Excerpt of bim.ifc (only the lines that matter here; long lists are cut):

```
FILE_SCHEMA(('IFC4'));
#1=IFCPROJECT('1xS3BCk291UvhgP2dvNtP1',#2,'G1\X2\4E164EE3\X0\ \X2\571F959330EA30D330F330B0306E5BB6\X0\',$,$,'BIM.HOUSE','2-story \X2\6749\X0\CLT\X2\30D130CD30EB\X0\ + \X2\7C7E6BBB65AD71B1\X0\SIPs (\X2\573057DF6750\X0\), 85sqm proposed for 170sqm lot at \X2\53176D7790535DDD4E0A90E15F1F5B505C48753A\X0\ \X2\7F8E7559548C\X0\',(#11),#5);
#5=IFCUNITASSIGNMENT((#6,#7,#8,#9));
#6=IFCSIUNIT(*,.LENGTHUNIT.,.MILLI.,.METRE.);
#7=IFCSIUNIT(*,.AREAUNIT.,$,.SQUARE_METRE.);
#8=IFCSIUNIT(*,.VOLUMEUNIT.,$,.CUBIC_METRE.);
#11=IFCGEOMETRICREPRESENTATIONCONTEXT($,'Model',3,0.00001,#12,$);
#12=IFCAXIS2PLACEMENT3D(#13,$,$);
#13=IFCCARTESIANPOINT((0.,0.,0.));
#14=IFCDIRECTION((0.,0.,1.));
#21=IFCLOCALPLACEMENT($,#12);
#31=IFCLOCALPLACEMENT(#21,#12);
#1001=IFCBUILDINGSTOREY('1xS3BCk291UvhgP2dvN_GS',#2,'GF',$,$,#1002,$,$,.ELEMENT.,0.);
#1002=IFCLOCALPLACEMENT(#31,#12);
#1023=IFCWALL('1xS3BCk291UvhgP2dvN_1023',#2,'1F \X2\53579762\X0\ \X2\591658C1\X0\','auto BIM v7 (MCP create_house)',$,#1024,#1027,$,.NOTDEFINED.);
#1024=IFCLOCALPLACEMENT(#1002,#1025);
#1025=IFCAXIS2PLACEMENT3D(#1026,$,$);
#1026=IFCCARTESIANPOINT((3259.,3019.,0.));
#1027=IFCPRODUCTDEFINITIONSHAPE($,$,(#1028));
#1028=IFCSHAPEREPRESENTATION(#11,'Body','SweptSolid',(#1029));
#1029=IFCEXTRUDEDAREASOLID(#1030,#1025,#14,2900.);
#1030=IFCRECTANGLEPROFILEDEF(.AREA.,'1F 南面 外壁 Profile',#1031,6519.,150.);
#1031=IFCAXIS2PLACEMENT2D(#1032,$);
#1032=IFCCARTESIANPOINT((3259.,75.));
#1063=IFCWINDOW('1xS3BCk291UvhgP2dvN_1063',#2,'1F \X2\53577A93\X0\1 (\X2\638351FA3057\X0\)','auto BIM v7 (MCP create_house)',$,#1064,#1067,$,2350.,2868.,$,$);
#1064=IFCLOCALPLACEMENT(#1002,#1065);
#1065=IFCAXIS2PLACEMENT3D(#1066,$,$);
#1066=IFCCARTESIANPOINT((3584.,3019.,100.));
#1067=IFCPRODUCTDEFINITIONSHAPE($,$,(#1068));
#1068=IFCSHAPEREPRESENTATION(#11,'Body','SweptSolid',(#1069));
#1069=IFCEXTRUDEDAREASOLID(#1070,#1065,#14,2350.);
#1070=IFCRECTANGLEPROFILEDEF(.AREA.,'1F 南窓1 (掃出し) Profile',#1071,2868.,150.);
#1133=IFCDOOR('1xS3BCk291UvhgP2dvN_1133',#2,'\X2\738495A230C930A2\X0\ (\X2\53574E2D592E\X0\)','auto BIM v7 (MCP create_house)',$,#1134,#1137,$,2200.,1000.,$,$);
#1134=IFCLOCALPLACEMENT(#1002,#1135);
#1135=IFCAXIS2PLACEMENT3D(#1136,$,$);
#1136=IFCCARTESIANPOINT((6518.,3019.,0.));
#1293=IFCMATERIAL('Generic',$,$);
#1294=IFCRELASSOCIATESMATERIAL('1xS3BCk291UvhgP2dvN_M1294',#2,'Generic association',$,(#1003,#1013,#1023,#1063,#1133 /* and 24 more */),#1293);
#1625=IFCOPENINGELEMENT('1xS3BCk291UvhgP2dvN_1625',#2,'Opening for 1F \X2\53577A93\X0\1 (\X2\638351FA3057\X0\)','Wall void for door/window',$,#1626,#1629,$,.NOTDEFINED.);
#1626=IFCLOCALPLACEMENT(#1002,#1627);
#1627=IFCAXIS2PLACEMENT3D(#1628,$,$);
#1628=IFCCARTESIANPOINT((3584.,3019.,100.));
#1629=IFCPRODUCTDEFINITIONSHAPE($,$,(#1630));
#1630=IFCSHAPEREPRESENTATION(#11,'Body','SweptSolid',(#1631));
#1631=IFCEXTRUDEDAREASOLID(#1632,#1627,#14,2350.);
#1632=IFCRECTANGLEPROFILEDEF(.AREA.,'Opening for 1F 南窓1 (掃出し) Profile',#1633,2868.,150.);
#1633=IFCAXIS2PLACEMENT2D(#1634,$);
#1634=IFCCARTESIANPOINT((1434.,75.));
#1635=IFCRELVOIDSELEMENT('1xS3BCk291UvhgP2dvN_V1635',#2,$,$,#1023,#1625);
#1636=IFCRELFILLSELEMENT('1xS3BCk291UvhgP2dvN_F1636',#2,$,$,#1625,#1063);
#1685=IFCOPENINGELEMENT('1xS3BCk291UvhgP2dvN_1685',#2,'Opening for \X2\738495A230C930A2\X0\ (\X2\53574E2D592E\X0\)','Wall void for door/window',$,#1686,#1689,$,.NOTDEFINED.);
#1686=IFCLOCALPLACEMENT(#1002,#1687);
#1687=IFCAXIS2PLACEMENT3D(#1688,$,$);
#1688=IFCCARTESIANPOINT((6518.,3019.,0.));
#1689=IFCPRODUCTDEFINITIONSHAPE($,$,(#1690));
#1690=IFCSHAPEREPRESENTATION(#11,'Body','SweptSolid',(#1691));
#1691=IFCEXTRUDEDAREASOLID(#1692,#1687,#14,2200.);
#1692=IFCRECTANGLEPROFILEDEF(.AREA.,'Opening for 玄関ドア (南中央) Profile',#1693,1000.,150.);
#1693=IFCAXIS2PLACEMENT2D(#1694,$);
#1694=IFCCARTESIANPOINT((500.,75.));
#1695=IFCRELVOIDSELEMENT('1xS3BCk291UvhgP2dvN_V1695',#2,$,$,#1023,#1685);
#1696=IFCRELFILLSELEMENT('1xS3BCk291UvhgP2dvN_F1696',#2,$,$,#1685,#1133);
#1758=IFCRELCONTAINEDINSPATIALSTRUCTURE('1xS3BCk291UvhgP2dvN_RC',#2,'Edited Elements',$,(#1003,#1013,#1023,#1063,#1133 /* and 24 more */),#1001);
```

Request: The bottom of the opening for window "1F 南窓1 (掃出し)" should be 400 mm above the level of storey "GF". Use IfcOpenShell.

```python
import numpy as np
import ifcopenshell
import ifcopenshell.api.geometry
import ifcopenshell.geom
import ifcopenshell.util.element
import ifcopenshell.util.placement
import ifcopenshell.util.shape
import ifcopenshell.util.unit

model = ifcopenshell.open("bim.ifc")
unit_scale = ifcopenshell.util.unit.calculate_unit_scale(model)

window = model.by_guid("1xS3BCk291UvhgP2dvN_1063")
opening = window.FillsVoids[0].RelatingOpeningElement
storey = ifcopenshell.util.element.get_container(window, ifc_class="IfcBuildingStorey")
level = ifcopenshell.util.placement.get_local_placement(storey.ObjectPlacement)[2, 3]

# The opening's origin need not be at the sill, so measure its lowest point.
shape = ifcopenshell.geom.create_shape(ifcopenshell.geom.settings(), opening)
bottom = ifcopenshell.util.shape.get_shape_bottom_elevation(shape, shape.geometry) / unit_scale
dz = level + 400.0 - bottom

shift = np.array([0.0, 0.0, dz])
# The window is not placed relative to its opening, so move both.
for product in (opening, window):
    matrix = ifcopenshell.util.placement.get_local_placement(product.ObjectPlacement)
    matrix[:3, 3] += shift
    ifcopenshell.api.geometry.edit_object_placement(model, product=product, matrix=matrix, is_si=False)

print(f"moved by {dz * unit_scale:+.3f} m")

model.write("bim_v2.ifc")
```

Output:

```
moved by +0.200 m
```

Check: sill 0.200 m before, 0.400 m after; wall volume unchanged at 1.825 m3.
